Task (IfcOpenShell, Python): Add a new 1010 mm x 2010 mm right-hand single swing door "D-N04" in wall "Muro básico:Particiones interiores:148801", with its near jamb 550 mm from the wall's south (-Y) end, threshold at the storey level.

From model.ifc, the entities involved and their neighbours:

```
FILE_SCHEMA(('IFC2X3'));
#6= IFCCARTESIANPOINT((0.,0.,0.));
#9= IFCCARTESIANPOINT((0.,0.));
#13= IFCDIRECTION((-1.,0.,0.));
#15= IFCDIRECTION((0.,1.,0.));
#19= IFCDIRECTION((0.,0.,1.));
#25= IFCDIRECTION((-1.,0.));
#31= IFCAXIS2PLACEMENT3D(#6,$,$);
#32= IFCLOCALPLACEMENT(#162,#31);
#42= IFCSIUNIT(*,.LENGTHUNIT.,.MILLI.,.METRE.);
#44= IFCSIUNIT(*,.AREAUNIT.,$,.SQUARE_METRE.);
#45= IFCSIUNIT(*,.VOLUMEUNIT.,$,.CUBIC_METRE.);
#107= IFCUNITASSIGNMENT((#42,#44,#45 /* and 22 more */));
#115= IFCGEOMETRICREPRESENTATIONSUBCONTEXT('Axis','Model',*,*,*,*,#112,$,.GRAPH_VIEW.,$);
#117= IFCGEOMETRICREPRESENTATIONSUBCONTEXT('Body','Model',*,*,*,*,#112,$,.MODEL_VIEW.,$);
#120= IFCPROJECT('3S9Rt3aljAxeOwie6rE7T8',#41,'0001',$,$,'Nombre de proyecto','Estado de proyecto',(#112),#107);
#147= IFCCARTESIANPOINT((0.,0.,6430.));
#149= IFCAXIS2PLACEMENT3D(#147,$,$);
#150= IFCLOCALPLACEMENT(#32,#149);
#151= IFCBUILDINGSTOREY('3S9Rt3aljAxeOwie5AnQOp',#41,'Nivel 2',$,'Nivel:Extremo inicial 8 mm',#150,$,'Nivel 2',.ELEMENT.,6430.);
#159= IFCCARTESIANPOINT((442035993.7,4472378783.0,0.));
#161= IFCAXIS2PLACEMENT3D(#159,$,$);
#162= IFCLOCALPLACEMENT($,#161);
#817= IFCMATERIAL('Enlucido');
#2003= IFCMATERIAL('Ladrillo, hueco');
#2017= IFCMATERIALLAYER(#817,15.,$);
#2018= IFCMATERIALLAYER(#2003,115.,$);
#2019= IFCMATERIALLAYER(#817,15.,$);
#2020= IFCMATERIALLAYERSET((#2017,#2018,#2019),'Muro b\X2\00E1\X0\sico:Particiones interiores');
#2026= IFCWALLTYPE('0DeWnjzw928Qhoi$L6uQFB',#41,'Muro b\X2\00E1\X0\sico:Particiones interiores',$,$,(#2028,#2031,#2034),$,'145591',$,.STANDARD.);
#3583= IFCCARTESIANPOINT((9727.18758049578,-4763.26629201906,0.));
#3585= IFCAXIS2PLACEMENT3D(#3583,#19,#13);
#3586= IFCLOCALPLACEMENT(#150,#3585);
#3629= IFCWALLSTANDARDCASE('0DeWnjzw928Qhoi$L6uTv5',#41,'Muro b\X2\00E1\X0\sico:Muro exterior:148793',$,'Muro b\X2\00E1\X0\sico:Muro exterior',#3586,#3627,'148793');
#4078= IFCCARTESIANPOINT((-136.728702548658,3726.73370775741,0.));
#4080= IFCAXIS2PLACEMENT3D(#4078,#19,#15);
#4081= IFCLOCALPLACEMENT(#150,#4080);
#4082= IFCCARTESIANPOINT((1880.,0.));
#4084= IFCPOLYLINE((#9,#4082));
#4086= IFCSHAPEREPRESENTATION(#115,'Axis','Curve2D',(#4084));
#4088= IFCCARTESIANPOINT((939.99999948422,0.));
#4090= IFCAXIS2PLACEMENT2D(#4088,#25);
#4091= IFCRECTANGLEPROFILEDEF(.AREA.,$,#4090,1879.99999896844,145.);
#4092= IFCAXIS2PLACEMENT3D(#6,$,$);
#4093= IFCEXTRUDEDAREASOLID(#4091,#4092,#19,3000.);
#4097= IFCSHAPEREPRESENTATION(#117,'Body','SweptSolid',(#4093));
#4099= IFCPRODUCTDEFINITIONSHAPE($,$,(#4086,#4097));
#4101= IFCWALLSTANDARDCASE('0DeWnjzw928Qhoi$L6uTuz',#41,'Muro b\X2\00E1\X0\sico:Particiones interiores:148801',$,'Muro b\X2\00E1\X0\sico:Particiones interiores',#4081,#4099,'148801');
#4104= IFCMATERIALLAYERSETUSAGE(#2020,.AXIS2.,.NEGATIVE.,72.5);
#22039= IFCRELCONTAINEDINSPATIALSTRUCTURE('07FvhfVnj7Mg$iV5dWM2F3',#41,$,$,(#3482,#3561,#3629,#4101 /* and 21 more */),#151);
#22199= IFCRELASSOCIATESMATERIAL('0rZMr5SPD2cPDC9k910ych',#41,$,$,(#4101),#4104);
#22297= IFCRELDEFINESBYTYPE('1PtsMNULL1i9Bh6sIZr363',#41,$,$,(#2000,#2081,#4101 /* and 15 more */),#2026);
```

```python
import numpy as np
import ifcopenshell
import ifcopenshell.api.feature
import ifcopenshell.api.geometry
import ifcopenshell.api.root
import ifcopenshell.api.spatial
import ifcopenshell.api.type
import ifcopenshell.geom
import ifcopenshell.util.element
import ifcopenshell.util.placement
import ifcopenshell.util.representation
import ifcopenshell.util.shape
import ifcopenshell.util.unit

model = ifcopenshell.open("model.ifc")
unit_scale = ifcopenshell.util.unit.calculate_unit_scale(model)
settings = ifcopenshell.geom.settings()


def volume(element):
    """Net volume in cubic metres, openings subtracted."""
    shape = ifcopenshell.geom.create_shape(settings, element)
    return ifcopenshell.util.shape.get_volume(shape.geometry)


wall = model.by_guid("0DeWnjzw928Qhoi$L6uTuz")
storey = ifcopenshell.util.element.get_container(wall, ifc_class="IfcBuildingStorey")
context = ifcopenshell.util.representation.get_context(model, "Model", "Body", "MODEL_VIEW")
before = volume(wall)

width, height, from_end, sill = 1.01, 2.01, 0.55, 0.0  # metres

# The wall runs along its own X axis, and the end named is its -X end.
wall_shape = ifcopenshell.geom.create_shape(settings, wall)
x, y, z = ifcopenshell.util.shape.get_vertices(wall_shape.geometry).T
start = x.min() + from_end
face, thickness = float(y.min()), float(y.max() - y.min())
wall_matrix = ifcopenshell.util.placement.get_local_placement(wall.ObjectPlacement)
level = ifcopenshell.util.placement.get_local_placement(storey.ObjectPlacement)[2, 3]


def in_wall(x, y):
    """Placement at x, y metres in the wall's axes, at sill height."""
    matrix = wall_matrix.copy()
    matrix[:, 3] = wall_matrix @ np.array([x / unit_scale, y / unit_scale, 0.0, 1.0])
    matrix[2, 3] = level + sill / unit_scale
    return matrix


# Opening: a box that overshoots both wall faces by 50 mm.
opening = ifcopenshell.api.root.create_entity(model, ifc_class="IfcOpeningElement")
box = ifcopenshell.api.geometry.add_wall_representation(
    model, context=context, length=width, height=height, thickness=thickness + 0.1
)
ifcopenshell.api.geometry.assign_representation(model, product=opening, representation=box)
ifcopenshell.api.geometry.edit_object_placement(model, product=opening, matrix=in_wall(start, face - 0.05), is_si=False)
ifcopenshell.api.feature.add_feature(model, feature=opening, element=wall)

door = ifcopenshell.api.root.create_entity(model, ifc_class="IfcDoor", name="D-N04")
door.OverallWidth, door.OverallHeight = width / unit_scale, height / unit_scale
body = ifcopenshell.api.geometry.add_door_representation(
    model,
    context=context,
    overall_width=door.OverallWidth,
    overall_height=door.OverallHeight,
    operation_type="SINGLE_SWING_RIGHT",
    lining_properties={"LiningDepth": thickness / unit_scale, "ThresholdDepth": thickness / unit_scale},
)
ifcopenshell.api.geometry.assign_representation(model, product=door, representation=body)
ifcopenshell.api.spatial.assign_container(model, products=[door], relating_structure=storey)
fills = ifcopenshell.api.feature.add_filling(model, opening=opening, element=door)
fills.OwnerHistory = door.OwnerHistory  # required in IFC2X3

# IFC2X3 keeps the operation on the door style.
style = ifcopenshell.api.root.create_entity(model, ifc_class="IfcDoorStyle", name="D-N04")
style.OperationType, style.ConstructionType = "SINGLE_SWING_RIGHT", "NOTDEFINED"
style.ParameterTakesPrecedence = style.Sizeable = False
ifcopenshell.api.type.assign_type(model, related_objects=[door], relating_type=style)

# The lining spans the wall, so the door starts at the wall face.
ifcopenshell.api.geometry.edit_object_placement(model, product=door, matrix=in_wall(start, face), is_si=False)

after = volume(wall)

print(f"wall volume {before:.3f} -> {after:.3f} m3")

model.write("model_updated.ifc")
```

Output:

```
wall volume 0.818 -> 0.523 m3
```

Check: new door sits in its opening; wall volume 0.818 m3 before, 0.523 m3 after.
